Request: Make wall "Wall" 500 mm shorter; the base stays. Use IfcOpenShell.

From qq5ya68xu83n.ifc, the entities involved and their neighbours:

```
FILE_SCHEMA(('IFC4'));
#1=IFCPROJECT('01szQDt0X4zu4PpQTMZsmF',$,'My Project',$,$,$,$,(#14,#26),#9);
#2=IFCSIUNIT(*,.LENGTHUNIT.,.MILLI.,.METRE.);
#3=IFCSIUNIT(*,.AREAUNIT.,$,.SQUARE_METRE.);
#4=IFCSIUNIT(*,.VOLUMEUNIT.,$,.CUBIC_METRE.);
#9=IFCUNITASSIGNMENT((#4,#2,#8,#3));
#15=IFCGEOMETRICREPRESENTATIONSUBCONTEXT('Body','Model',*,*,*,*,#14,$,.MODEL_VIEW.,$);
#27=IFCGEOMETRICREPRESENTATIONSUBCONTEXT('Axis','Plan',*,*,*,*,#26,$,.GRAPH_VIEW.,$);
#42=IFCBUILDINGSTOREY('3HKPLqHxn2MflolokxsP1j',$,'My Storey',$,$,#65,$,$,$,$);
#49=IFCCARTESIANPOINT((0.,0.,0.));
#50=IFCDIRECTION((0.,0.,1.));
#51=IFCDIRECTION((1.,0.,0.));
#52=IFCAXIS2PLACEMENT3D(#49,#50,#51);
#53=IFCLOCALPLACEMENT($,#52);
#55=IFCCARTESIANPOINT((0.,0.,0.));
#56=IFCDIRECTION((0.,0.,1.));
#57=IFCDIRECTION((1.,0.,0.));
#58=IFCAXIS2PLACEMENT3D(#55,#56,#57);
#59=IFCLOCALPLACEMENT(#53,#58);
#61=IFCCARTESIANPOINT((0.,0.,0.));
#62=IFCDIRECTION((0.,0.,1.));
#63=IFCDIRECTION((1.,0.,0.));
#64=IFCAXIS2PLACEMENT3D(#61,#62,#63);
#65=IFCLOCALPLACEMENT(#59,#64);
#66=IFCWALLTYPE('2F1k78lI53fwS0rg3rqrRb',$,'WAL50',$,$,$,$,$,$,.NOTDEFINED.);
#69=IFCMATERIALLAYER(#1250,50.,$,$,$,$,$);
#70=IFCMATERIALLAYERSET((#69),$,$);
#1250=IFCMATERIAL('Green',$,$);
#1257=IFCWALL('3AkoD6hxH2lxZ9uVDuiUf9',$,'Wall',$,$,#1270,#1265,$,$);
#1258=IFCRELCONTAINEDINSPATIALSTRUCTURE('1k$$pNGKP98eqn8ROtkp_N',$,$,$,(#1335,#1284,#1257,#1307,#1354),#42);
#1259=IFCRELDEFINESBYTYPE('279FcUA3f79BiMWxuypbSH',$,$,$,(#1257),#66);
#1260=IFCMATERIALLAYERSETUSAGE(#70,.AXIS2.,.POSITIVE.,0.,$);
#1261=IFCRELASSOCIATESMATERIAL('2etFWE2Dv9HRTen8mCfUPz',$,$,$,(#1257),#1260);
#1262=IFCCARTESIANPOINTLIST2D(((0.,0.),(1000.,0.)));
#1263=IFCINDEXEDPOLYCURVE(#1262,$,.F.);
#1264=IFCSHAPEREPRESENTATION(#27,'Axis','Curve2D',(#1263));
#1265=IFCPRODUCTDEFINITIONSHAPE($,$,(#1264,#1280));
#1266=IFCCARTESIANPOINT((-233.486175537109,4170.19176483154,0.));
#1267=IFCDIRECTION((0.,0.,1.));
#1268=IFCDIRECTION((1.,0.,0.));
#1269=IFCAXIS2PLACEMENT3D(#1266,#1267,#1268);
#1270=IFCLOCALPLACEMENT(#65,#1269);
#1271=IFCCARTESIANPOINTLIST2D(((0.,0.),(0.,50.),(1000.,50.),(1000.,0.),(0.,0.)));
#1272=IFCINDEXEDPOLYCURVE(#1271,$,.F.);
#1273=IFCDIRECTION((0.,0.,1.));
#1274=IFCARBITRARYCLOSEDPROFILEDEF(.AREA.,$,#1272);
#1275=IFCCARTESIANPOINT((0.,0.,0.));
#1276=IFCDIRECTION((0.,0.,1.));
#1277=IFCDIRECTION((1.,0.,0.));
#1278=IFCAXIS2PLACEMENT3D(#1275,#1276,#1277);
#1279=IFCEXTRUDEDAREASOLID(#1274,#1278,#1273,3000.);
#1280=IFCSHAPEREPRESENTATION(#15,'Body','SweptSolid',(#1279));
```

```python
import ifcopenshell
import ifcopenshell.geom
import ifcopenshell.util.representation
import ifcopenshell.util.shape

model = ifcopenshell.open("qq5ya68xu83n.ifc")
settings = ifcopenshell.geom.settings()


def volume(element):
    """Net volume in cubic metres, openings subtracted."""
    shape = ifcopenshell.geom.create_shape(settings, element)
    return ifcopenshell.util.shape.get_volume(shape.geometry)


wall = model.by_id(1257)
before = volume(wall)

body = ifcopenshell.util.representation.get_representation(wall, "Model", "Body")
solid = body.Items[0]
old_height = solid.Depth
solid.Depth -= 500.0
after = volume(wall)

print(f"height {old_height:g} -> {solid.Depth:g}, volume {before:.3f} -> {after:.3f} m3")

model.write("qq5ya68xu83n_v2.ifc")
```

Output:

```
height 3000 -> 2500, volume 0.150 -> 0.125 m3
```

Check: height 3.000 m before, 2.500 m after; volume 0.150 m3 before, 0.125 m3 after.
